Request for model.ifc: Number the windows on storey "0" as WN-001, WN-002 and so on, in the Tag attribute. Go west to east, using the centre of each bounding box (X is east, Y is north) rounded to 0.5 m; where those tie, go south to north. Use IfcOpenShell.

First a look at what the model holds.

```python
import ifcopenshell
import ifcopenshell.util.element
import ifcopenshell.util.placement

model = ifcopenshell.open("model.ifc")
print(model.schema)
storey = next(s for s in model.by_type("IfcBuildingStorey") if s.Name == "0")
windows = [e for e in ifcopenshell.util.element.get_decomposition(storey) if e.is_a("IfcWindow")]
for e in sorted(windows, key=lambda e: e.id()):
    origin = ifcopenshell.util.placement.get_local_placement(e.ObjectPlacement)[:3, 3]
    print(e.id(), e.Tag, e.Name, origin.round(2) + 0.0, sep=" | ")
```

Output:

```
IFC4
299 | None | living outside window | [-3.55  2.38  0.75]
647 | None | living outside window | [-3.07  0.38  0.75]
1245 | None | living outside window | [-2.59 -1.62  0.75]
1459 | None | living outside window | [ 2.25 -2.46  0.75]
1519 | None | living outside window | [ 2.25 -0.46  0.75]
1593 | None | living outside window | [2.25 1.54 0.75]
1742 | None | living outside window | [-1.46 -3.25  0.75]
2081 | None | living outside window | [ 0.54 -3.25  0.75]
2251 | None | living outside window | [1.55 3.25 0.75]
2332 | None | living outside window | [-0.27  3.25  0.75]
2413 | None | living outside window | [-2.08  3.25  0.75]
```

```python
import ifcopenshell
import ifcopenshell.geom
import ifcopenshell.util.element
import ifcopenshell.util.shape

model = ifcopenshell.open("model.ifc")
settings = ifcopenshell.geom.settings()
settings.set("use-world-coords", True)


def centre(element):
    shape = ifcopenshell.geom.create_shape(settings, element)
    return ifcopenshell.util.shape.get_bbox_centroid(shape.geometry)


storey = next(s for s in model.by_type("IfcBuildingStorey") if s.Name == "0")
windows = [e for e in ifcopenshell.util.element.get_decomposition(storey) if e.is_a("IfcWindow")]

# Insertion points can sit at a corner or the storey origin, so sort by the geometry (in metres).
centres = {e: centre(e) for e in windows}
windows.sort(key=lambda e: (round(centres[e][0] / 0.5), centres[e][1]))

for i, e in enumerate(windows, start=1):
    number = f"WN-0{i:02d}"
    e.Tag = number
    print(e.id(), number)

model.write("model_v2.ifc")
```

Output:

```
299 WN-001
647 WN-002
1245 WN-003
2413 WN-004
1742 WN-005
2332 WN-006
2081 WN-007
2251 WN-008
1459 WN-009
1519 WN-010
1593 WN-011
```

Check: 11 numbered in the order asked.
